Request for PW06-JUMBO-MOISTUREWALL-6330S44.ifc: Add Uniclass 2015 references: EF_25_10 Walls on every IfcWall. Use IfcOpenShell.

First a look at what the model holds.

```python
import ifcopenshell

model = ifcopenshell.open("PW06-JUMBO-MOISTUREWALL-6330S44.ifc")
print(model.schema)
print("classifications:", [c.Name for c in model.by_type("IfcClassification")])
for ifc_class in ("IfcDoor", "IfcRoof", "IfcStair", "IfcWall", "IfcWindow"):
    print(ifc_class, len(model.by_type(ifc_class)))
```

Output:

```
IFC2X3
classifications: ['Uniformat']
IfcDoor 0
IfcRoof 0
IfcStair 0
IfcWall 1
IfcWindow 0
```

```python
import ifcopenshell
import ifcopenshell.api.classification

model = ifcopenshell.open("PW06-JUMBO-MOISTUREWALL-6330S44.ifc")

# IFC2X3 requires Source and Edition and has no link from the project to the system.
system = model.create_entity("IfcClassification", Source="NBS", Edition="2015", Name="Uniclass 2015")

codes = {
    "IfcWall": ("EF_25_10", "Walls"),
}
for ifc_class, (code, name) in codes.items():
    products = model.by_type(ifc_class)
    ifcopenshell.api.classification.add_reference(
        model, products=products, classification=system, identification=code, name=name
    )
    print(code, len(products))

model.write("PW06-JUMBO-MOISTUREWALL-6330S44_edited.ifc")
```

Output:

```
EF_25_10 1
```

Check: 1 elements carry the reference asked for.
